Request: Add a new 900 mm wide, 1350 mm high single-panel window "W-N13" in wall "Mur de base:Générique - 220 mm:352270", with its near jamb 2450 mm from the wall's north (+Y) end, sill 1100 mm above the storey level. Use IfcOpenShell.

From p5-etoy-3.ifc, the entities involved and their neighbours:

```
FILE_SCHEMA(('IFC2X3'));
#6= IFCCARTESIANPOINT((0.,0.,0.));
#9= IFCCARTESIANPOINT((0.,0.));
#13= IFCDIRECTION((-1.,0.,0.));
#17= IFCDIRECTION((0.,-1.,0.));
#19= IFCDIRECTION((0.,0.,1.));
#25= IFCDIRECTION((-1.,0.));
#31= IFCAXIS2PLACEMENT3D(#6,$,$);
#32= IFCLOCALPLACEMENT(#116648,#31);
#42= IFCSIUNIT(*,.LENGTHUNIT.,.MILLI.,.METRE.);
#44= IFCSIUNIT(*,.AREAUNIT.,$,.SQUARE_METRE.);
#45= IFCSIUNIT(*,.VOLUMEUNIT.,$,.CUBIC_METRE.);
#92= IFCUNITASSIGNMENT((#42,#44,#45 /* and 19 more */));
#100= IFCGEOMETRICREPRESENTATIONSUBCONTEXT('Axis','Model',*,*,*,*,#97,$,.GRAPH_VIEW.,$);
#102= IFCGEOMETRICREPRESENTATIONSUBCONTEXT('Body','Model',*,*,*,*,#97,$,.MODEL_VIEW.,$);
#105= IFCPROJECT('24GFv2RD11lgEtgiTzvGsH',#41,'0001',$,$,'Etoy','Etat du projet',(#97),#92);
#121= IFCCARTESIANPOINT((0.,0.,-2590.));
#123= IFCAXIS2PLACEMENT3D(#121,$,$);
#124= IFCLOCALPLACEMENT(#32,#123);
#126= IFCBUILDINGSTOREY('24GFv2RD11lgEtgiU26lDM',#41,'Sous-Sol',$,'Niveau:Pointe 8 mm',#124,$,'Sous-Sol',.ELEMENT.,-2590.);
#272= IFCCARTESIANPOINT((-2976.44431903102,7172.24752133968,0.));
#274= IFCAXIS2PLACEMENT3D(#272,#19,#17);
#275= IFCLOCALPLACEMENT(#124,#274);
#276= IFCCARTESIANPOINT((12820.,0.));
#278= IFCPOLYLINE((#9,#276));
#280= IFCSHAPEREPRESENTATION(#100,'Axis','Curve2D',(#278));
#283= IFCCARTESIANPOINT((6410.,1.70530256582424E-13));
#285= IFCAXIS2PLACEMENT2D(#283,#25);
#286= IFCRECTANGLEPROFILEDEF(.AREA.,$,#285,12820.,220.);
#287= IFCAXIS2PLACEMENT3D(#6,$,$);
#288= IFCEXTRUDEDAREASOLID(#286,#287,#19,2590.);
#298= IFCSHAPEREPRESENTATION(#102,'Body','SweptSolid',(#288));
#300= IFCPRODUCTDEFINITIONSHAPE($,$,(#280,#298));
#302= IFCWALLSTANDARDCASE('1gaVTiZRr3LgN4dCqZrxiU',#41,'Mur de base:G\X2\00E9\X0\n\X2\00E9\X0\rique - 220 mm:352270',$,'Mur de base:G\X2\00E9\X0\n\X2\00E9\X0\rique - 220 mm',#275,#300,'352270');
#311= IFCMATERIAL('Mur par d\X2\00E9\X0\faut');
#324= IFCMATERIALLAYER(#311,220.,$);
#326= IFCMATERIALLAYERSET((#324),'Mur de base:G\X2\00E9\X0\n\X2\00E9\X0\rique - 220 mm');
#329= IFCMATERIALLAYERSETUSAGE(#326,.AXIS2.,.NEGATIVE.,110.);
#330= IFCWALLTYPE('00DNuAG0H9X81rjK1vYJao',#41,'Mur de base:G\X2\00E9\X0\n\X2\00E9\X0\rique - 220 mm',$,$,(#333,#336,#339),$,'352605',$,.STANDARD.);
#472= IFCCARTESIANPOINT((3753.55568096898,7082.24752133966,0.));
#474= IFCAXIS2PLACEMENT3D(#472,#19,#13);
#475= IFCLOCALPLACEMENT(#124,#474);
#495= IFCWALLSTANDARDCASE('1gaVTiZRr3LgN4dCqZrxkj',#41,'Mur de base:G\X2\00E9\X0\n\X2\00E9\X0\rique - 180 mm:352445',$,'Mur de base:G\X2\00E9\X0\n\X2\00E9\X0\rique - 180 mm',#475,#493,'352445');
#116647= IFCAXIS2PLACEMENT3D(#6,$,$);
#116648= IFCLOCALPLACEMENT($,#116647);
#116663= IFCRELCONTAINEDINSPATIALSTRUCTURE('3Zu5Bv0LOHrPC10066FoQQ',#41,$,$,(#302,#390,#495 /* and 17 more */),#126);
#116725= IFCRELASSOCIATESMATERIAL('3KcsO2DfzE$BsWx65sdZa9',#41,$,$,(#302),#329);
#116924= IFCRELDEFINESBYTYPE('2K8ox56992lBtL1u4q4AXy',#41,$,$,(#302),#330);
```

```python
import numpy as np
import ifcopenshell
import ifcopenshell.api.feature
import ifcopenshell.api.geometry
import ifcopenshell.api.root
import ifcopenshell.api.spatial
import ifcopenshell.api.type
import ifcopenshell.geom
import ifcopenshell.util.element
import ifcopenshell.util.placement
import ifcopenshell.util.representation
import ifcopenshell.util.shape
import ifcopenshell.util.unit

model = ifcopenshell.open("p5-etoy-3.ifc")
unit_scale = ifcopenshell.util.unit.calculate_unit_scale(model)
settings = ifcopenshell.geom.settings()


def volume(element):
    """Net volume in cubic metres, openings subtracted."""
    shape = ifcopenshell.geom.create_shape(settings, element)
    return ifcopenshell.util.shape.get_volume(shape.geometry)


wall = model.by_guid("1gaVTiZRr3LgN4dCqZrxiU")
storey = ifcopenshell.util.element.get_container(wall, ifc_class="IfcBuildingStorey")
context = ifcopenshell.util.representation.get_context(model, "Model", "Body", "MODEL_VIEW")
before = volume(wall)

width, height, from_end, sill = 0.9, 1.35, 2.45, 1.1  # metres

# The wall runs along its own X axis, and the end named is its -X end.
wall_shape = ifcopenshell.geom.create_shape(settings, wall)
x, y, z = ifcopenshell.util.shape.get_vertices(wall_shape.geometry).T
start = x.min() + from_end
face, thickness = float(y.min()), float(y.max() - y.min())
wall_matrix = ifcopenshell.util.placement.get_local_placement(wall.ObjectPlacement)
level = ifcopenshell.util.placement.get_local_placement(storey.ObjectPlacement)[2, 3]


def in_wall(x, y):
    """Placement at x, y metres in the wall's axes, at sill height."""
    matrix = wall_matrix.copy()
    matrix[:, 3] = wall_matrix @ np.array([x / unit_scale, y / unit_scale, 0.0, 1.0])
    matrix[2, 3] = level + sill / unit_scale
    return matrix


# Opening: a box that overshoots both wall faces by 50 mm.
opening = ifcopenshell.api.root.create_entity(model, ifc_class="IfcOpeningElement")
box = ifcopenshell.api.geometry.add_wall_representation(
    model, context=context, length=width, height=height, thickness=thickness + 0.1
)
ifcopenshell.api.geometry.assign_representation(model, product=opening, representation=box)
ifcopenshell.api.geometry.edit_object_placement(model, product=opening, matrix=in_wall(start, face - 0.05), is_si=False)
ifcopenshell.api.feature.add_feature(model, feature=opening, element=wall)

window = ifcopenshell.api.root.create_entity(model, ifc_class="IfcWindow", name="W-N13")
window.OverallWidth, window.OverallHeight = width / unit_scale, height / unit_scale
body = ifcopenshell.api.geometry.add_window_representation(
    model,
    context=context,
    overall_width=window.OverallWidth,
    overall_height=window.OverallHeight,
    partition_type="SINGLE_PANEL",
)
ifcopenshell.api.geometry.assign_representation(model, product=window, representation=body)
ifcopenshell.api.spatial.assign_container(model, products=[window], relating_structure=storey)
fills = ifcopenshell.api.feature.add_filling(model, opening=opening, element=window)
fills.OwnerHistory = window.OwnerHistory  # required in IFC2X3

# IFC2X3 keeps the operation on the window style.
style = ifcopenshell.api.root.create_entity(model, ifc_class="IfcWindowStyle", name="W-N13")
style.OperationType, style.ConstructionType = "SINGLE_PANEL", "NOTDEFINED"
style.ParameterTakesPrecedence = style.Sizeable = False
ifcopenshell.api.type.assign_type(model, related_objects=[window], relating_type=style)

# Centre the window in the wall's thickness.
ifcopenshell.api.geometry.edit_object_placement(model, product=window, matrix=in_wall(start, face), is_si=False)
window_shape = ifcopenshell.geom.create_shape(settings, window)
depth = ifcopenshell.util.shape.get_vertices(window_shape.geometry)[:, 1]
offset = face + thickness / 2 - (depth.min() + depth.max()) / 2
ifcopenshell.api.geometry.edit_object_placement(model, product=window, matrix=in_wall(start, offset), is_si=False)

after = volume(wall)

print(f"wall volume {before:.3f} -> {after:.3f} m3")

model.write("p5-etoy-3_edited.ifc")
```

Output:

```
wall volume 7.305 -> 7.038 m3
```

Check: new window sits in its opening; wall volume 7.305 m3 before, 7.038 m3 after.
